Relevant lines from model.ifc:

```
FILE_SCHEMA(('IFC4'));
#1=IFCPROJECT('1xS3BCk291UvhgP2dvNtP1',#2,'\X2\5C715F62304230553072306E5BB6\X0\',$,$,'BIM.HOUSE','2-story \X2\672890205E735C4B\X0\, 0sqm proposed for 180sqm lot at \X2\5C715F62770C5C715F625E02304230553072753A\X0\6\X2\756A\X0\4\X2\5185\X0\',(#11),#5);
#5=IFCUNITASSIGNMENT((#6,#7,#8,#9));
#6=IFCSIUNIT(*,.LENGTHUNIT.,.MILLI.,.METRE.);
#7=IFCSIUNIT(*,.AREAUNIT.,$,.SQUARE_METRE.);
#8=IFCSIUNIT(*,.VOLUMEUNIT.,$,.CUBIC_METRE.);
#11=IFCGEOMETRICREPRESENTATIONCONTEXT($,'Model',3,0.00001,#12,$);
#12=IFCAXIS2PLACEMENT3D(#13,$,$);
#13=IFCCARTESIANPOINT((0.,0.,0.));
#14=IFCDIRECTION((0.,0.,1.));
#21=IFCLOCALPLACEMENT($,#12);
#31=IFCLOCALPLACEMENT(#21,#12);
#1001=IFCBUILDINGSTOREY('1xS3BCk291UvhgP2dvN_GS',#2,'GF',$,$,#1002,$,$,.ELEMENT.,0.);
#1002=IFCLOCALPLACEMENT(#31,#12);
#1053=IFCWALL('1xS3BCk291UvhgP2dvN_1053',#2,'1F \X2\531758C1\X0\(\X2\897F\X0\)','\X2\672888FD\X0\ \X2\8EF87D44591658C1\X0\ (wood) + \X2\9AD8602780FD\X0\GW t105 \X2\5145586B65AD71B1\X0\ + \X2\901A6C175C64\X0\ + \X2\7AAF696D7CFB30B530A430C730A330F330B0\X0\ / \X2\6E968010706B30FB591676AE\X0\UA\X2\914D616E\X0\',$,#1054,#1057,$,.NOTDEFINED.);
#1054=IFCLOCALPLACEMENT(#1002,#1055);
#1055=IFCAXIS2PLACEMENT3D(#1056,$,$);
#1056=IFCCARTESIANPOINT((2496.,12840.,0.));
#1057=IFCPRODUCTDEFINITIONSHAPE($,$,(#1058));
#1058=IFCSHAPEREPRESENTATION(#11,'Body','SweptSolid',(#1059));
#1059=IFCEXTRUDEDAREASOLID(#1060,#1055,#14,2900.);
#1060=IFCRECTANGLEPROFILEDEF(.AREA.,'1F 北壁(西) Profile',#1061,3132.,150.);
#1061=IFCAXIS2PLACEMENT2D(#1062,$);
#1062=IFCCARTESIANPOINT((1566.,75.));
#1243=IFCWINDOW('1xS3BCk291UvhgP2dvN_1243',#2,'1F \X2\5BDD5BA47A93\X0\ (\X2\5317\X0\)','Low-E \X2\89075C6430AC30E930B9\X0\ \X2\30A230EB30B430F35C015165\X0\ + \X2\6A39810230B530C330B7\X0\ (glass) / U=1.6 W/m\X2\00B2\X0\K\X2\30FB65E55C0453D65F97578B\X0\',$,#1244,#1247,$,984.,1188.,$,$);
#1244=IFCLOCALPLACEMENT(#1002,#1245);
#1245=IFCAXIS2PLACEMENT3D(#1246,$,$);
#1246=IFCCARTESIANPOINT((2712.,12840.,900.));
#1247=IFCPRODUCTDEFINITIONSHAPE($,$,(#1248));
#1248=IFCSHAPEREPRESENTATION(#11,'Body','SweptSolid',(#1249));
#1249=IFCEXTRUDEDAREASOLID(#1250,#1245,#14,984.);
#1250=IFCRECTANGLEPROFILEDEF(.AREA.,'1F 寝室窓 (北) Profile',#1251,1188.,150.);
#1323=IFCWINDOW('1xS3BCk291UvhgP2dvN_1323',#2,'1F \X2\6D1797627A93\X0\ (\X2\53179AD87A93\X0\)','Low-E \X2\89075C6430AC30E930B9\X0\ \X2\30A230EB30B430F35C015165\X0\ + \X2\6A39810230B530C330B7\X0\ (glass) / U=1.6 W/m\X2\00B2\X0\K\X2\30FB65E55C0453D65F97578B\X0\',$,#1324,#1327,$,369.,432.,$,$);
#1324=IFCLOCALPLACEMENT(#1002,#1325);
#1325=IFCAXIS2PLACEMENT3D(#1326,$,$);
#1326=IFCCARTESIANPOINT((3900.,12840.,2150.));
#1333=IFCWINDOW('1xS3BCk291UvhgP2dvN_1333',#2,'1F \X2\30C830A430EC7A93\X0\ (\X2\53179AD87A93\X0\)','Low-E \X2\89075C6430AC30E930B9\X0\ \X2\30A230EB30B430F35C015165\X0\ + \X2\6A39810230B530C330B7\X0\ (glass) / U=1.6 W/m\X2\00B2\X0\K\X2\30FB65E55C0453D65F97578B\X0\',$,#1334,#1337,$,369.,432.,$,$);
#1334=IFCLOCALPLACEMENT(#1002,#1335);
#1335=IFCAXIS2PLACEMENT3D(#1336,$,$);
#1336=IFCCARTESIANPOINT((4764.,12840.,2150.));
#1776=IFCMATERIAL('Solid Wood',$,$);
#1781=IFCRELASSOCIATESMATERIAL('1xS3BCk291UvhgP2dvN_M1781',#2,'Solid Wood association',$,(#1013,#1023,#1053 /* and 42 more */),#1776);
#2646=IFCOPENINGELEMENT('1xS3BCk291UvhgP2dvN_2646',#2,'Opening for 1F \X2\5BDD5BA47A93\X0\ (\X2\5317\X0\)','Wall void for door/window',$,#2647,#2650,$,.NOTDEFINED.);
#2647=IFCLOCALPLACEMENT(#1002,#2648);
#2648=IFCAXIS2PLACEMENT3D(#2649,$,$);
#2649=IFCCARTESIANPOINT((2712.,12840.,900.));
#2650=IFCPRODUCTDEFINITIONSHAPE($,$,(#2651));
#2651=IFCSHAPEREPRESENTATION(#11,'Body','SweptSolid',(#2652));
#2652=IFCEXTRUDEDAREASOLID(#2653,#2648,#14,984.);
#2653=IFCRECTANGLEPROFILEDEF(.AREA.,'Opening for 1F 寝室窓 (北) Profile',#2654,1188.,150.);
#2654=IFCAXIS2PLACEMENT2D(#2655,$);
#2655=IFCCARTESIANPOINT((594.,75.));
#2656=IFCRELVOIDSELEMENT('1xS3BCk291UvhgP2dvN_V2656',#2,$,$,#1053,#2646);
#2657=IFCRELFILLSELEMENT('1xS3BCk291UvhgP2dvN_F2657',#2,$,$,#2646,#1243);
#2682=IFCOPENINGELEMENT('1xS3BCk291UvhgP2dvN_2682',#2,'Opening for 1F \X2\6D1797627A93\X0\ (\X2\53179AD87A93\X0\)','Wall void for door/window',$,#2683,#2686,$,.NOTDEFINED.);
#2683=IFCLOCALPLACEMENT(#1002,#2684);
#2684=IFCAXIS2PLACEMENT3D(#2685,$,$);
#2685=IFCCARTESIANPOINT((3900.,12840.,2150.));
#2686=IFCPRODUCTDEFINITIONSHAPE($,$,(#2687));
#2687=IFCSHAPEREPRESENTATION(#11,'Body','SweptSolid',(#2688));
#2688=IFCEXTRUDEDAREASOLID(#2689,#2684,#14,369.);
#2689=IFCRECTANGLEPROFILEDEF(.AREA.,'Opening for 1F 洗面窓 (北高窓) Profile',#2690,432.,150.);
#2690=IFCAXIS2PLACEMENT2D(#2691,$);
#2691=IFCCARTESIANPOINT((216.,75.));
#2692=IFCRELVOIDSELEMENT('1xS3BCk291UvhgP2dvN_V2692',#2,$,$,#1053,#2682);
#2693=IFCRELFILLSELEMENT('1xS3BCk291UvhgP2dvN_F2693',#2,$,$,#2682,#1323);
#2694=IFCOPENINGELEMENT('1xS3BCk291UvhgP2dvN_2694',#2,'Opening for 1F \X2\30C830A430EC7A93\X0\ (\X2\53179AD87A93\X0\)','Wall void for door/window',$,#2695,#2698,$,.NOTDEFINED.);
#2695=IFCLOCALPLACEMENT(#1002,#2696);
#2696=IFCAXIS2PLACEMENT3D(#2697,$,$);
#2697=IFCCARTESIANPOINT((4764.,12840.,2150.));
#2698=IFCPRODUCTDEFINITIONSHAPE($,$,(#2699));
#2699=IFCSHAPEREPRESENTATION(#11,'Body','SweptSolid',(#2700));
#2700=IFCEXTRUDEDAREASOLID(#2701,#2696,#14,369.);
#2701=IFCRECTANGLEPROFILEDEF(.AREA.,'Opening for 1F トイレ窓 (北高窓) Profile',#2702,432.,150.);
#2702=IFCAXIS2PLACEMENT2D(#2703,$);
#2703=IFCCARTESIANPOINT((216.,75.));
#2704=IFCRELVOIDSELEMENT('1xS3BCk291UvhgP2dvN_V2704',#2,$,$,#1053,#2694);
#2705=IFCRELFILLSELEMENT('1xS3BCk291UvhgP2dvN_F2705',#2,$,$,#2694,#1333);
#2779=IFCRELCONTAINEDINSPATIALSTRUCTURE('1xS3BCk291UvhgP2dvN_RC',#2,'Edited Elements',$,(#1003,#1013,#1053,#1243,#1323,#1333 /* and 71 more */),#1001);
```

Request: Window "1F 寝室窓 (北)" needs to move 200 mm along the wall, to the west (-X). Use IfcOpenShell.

```python
import ifcopenshell
import ifcopenshell.api.geometry
import ifcopenshell.util.placement
import ifcopenshell.util.unit

model = ifcopenshell.open("model.ifc")
unit_scale = ifcopenshell.util.unit.calculate_unit_scale(model)

window = model.by_id(1243)
opening = window.FillsVoids[0].RelatingOpeningElement
wall = opening.VoidsElements[0].RelatingBuildingElement

wall_matrix = ifcopenshell.util.placement.get_local_placement(wall.ObjectPlacement)
shift = wall_matrix[:3, 0] * -0.2 / unit_scale
before = ifcopenshell.util.placement.get_local_placement(window.ObjectPlacement)[:3, 3].copy()

# The window is not placed relative to its opening, so move both.
for product in (opening, window):
    matrix = ifcopenshell.util.placement.get_local_placement(product.ObjectPlacement)
    matrix[:3, 3] += shift
    ifcopenshell.api.geometry.edit_object_placement(model, product=product, matrix=matrix, is_si=False)

after = ifcopenshell.util.placement.get_local_placement(window.ObjectPlacement)[:3, 3]
print("window moved by", (after - before).round(3) + 0.0)

model.write("model_v2.ifc")
```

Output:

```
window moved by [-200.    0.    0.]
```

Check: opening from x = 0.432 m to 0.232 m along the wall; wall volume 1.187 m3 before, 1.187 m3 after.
